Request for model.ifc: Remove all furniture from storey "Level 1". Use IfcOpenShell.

First a look at what the model holds.

```python
import ifcopenshell
import ifcopenshell.util.element

model = ifcopenshell.open("model.ifc")
print(model.schema)
storey = next(s for s in model.by_type("IfcBuildingStorey") if s.Name == "Level 1")
furniture = [e for e in ifcopenshell.util.element.get_decomposition(storey) if e.is_a("IfcFurnishingElement")]
seen = {}
for e in furniture:
    element_type = ifcopenshell.util.element.get_type(e)
    name = element_type.Name if element_type not in (None, e) else None
    seen[name] = seen.get(name, 0) + 1
for name, count in sorted(seen.items(), key=str):
    print(count, "x", name)
```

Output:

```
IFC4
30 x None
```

```python
import ifcopenshell
import ifcopenshell.api.root
import ifcopenshell.util.element

model = ifcopenshell.open("model.ifc")

storey = next(s for s in model.by_type("IfcBuildingStorey") if s.Name == "Level 1")
furniture = [e for e in ifcopenshell.util.element.get_decomposition(storey) if e.is_a("IfcFurnishingElement")]

for e in furniture:
    ifcopenshell.api.root.remove_product(model, product=e)
print(len(furniture), "removed")

model.write("model_edited.ifc")
```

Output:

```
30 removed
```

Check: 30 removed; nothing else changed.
